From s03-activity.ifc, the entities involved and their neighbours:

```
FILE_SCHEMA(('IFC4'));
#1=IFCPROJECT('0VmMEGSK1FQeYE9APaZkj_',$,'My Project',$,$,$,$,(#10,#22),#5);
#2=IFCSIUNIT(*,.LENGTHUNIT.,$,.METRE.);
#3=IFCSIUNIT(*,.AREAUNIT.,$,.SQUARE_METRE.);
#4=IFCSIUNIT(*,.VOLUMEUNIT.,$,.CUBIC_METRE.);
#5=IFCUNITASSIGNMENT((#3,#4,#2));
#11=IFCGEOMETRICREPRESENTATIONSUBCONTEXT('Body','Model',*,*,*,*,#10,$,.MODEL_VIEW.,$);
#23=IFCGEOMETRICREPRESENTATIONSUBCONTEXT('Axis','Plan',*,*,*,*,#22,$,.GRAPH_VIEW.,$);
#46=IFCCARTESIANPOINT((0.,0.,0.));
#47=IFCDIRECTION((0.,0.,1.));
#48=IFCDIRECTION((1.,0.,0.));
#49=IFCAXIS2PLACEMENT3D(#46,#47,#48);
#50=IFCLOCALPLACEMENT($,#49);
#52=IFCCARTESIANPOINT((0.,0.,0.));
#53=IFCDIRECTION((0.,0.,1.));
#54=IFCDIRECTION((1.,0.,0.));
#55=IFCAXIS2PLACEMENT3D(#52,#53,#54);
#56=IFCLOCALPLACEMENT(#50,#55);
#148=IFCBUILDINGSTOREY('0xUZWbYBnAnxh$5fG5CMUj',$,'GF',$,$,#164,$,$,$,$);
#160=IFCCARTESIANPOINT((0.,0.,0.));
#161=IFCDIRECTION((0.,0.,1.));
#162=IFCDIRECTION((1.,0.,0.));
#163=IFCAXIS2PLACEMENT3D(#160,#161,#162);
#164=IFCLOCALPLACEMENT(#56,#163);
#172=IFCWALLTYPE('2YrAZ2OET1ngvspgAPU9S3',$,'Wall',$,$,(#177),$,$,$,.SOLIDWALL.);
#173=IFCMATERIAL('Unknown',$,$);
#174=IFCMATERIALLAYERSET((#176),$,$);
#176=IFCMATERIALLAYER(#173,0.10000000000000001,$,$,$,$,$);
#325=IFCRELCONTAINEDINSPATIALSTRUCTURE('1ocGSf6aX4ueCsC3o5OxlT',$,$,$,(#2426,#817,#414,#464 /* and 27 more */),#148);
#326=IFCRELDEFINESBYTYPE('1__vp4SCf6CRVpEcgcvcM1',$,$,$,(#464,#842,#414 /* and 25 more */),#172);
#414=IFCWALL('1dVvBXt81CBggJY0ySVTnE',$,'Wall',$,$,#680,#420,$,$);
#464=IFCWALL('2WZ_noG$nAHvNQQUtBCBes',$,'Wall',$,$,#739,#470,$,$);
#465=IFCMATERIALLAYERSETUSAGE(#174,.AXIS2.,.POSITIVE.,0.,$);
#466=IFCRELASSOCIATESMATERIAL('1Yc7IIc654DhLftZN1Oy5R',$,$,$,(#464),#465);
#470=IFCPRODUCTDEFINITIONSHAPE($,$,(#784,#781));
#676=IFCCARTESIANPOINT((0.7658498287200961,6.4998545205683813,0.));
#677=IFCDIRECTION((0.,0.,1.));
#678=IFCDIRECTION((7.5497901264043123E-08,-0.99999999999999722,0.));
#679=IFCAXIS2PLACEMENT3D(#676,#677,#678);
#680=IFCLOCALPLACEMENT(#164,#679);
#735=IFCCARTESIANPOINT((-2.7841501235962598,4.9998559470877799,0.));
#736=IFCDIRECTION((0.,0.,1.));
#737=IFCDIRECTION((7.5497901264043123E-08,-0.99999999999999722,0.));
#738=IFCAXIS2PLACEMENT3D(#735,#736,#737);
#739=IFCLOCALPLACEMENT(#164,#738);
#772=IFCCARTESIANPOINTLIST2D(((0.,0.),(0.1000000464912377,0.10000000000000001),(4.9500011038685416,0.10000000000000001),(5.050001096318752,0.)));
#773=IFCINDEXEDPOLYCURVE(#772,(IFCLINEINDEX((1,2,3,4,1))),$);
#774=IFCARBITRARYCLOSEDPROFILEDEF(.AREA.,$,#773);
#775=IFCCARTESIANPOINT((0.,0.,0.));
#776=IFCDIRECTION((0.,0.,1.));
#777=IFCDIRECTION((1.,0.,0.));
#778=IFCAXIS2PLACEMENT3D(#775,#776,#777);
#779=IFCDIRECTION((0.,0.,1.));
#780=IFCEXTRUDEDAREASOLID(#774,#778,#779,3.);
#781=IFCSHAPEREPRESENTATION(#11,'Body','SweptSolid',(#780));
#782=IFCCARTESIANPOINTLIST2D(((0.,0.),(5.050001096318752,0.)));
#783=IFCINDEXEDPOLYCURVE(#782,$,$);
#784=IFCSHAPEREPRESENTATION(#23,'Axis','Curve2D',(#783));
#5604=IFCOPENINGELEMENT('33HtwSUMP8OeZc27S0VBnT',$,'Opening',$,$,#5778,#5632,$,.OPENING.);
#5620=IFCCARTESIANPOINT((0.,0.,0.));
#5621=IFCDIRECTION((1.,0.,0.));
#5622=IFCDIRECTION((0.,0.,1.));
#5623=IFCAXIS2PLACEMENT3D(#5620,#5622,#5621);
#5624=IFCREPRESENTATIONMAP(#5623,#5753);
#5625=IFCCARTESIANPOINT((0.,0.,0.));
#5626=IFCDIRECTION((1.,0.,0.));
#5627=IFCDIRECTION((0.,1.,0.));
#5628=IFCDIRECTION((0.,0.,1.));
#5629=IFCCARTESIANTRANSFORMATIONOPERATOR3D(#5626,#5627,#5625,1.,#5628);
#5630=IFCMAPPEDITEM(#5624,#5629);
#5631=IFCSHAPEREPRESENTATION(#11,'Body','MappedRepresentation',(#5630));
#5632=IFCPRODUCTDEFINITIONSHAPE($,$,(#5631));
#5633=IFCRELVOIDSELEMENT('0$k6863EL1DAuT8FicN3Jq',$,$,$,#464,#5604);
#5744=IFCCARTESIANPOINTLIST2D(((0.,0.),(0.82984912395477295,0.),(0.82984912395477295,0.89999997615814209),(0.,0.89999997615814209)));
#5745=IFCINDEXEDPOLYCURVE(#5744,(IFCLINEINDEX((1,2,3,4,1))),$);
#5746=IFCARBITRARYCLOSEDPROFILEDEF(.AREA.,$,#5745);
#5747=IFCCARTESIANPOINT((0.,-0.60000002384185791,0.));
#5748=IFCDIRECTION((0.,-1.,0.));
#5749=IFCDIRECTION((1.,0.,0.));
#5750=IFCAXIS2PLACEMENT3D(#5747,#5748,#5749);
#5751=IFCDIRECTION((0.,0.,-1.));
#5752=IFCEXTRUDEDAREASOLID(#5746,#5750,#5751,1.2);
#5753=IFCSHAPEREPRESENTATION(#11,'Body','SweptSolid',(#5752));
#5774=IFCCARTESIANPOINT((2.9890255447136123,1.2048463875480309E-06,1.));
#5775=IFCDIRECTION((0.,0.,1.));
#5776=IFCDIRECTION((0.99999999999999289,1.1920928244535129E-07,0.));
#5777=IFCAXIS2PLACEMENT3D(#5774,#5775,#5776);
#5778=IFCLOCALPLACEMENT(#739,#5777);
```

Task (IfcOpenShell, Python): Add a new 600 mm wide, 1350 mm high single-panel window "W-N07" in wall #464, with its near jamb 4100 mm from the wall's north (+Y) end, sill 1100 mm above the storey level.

```python
import numpy as np
import ifcopenshell
import ifcopenshell.api.feature
import ifcopenshell.api.geometry
import ifcopenshell.api.root
import ifcopenshell.api.spatial
import ifcopenshell.geom
import ifcopenshell.util.element
import ifcopenshell.util.placement
import ifcopenshell.util.representation
import ifcopenshell.util.shape
import ifcopenshell.util.unit

model = ifcopenshell.open("s03-activity.ifc")
unit_scale = ifcopenshell.util.unit.calculate_unit_scale(model)
settings = ifcopenshell.geom.settings()


def volume(element):
    """Net volume in cubic metres, openings subtracted."""
    shape = ifcopenshell.geom.create_shape(settings, element)
    return ifcopenshell.util.shape.get_volume(shape.geometry)


wall = model.by_guid("2WZ_noG$nAHvNQQUtBCBes")
storey = ifcopenshell.util.element.get_container(wall, ifc_class="IfcBuildingStorey")
context = ifcopenshell.util.representation.get_context(model, "Model", "Body", "MODEL_VIEW")
before = volume(wall)

width, height, from_end, sill = 0.6, 1.35, 4.1, 1.1  # metres

# The wall runs along its own X axis, and the end named is its -X end.
wall_shape = ifcopenshell.geom.create_shape(settings, wall)
x, y, z = ifcopenshell.util.shape.get_vertices(wall_shape.geometry).T
start = x.min() + from_end
face, thickness = float(y.min()), float(y.max() - y.min())
wall_matrix = ifcopenshell.util.placement.get_local_placement(wall.ObjectPlacement)
level = ifcopenshell.util.placement.get_local_placement(storey.ObjectPlacement)[2, 3]


def in_wall(x, y):
    """Placement at x, y metres in the wall's axes, at sill height."""
    matrix = wall_matrix.copy()
    matrix[:, 3] = wall_matrix @ np.array([x / unit_scale, y / unit_scale, 0.0, 1.0])
    matrix[2, 3] = level + sill / unit_scale
    return matrix


# Opening: a box that overshoots both wall faces by 50 mm.
opening = ifcopenshell.api.root.create_entity(model, ifc_class="IfcOpeningElement", predefined_type="OPENING")
box = ifcopenshell.api.geometry.add_wall_representation(
    model, context=context, length=width, height=height, thickness=thickness + 0.1
)
ifcopenshell.api.geometry.assign_representation(model, product=opening, representation=box)
ifcopenshell.api.geometry.edit_object_placement(model, product=opening, matrix=in_wall(start, face - 0.05), is_si=False)
ifcopenshell.api.feature.add_feature(model, feature=opening, element=wall)

window = ifcopenshell.api.root.create_entity(model, ifc_class="IfcWindow", name="W-N07", predefined_type="WINDOW")
window.OverallWidth, window.OverallHeight = width / unit_scale, height / unit_scale
window.PartitioningType = "SINGLE_PANEL"
body = ifcopenshell.api.geometry.add_window_representation(
    model,
    context=context,
    overall_width=window.OverallWidth,
    overall_height=window.OverallHeight,
    partition_type="SINGLE_PANEL",
)
ifcopenshell.api.geometry.assign_representation(model, product=window, representation=body)
ifcopenshell.api.spatial.assign_container(model, products=[window], relating_structure=storey)
ifcopenshell.api.feature.add_filling(model, opening=opening, element=window)

# Centre the window in the wall's thickness.
ifcopenshell.api.geometry.edit_object_placement(model, product=window, matrix=in_wall(start, face), is_si=False)
window_shape = ifcopenshell.geom.create_shape(settings, window)
depth = ifcopenshell.util.shape.get_vertices(window_shape.geometry)[:, 1]
offset = face + thickness / 2 - (depth.min() + depth.max()) / 2
ifcopenshell.api.geometry.edit_object_placement(model, product=window, matrix=in_wall(start, offset), is_si=False)

after = volume(wall)

print(f"wall volume {before:.3f} -> {after:.3f} m3")

model.write("s03-activity-out.ifc")
```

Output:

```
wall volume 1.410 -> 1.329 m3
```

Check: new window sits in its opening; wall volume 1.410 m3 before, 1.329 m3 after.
